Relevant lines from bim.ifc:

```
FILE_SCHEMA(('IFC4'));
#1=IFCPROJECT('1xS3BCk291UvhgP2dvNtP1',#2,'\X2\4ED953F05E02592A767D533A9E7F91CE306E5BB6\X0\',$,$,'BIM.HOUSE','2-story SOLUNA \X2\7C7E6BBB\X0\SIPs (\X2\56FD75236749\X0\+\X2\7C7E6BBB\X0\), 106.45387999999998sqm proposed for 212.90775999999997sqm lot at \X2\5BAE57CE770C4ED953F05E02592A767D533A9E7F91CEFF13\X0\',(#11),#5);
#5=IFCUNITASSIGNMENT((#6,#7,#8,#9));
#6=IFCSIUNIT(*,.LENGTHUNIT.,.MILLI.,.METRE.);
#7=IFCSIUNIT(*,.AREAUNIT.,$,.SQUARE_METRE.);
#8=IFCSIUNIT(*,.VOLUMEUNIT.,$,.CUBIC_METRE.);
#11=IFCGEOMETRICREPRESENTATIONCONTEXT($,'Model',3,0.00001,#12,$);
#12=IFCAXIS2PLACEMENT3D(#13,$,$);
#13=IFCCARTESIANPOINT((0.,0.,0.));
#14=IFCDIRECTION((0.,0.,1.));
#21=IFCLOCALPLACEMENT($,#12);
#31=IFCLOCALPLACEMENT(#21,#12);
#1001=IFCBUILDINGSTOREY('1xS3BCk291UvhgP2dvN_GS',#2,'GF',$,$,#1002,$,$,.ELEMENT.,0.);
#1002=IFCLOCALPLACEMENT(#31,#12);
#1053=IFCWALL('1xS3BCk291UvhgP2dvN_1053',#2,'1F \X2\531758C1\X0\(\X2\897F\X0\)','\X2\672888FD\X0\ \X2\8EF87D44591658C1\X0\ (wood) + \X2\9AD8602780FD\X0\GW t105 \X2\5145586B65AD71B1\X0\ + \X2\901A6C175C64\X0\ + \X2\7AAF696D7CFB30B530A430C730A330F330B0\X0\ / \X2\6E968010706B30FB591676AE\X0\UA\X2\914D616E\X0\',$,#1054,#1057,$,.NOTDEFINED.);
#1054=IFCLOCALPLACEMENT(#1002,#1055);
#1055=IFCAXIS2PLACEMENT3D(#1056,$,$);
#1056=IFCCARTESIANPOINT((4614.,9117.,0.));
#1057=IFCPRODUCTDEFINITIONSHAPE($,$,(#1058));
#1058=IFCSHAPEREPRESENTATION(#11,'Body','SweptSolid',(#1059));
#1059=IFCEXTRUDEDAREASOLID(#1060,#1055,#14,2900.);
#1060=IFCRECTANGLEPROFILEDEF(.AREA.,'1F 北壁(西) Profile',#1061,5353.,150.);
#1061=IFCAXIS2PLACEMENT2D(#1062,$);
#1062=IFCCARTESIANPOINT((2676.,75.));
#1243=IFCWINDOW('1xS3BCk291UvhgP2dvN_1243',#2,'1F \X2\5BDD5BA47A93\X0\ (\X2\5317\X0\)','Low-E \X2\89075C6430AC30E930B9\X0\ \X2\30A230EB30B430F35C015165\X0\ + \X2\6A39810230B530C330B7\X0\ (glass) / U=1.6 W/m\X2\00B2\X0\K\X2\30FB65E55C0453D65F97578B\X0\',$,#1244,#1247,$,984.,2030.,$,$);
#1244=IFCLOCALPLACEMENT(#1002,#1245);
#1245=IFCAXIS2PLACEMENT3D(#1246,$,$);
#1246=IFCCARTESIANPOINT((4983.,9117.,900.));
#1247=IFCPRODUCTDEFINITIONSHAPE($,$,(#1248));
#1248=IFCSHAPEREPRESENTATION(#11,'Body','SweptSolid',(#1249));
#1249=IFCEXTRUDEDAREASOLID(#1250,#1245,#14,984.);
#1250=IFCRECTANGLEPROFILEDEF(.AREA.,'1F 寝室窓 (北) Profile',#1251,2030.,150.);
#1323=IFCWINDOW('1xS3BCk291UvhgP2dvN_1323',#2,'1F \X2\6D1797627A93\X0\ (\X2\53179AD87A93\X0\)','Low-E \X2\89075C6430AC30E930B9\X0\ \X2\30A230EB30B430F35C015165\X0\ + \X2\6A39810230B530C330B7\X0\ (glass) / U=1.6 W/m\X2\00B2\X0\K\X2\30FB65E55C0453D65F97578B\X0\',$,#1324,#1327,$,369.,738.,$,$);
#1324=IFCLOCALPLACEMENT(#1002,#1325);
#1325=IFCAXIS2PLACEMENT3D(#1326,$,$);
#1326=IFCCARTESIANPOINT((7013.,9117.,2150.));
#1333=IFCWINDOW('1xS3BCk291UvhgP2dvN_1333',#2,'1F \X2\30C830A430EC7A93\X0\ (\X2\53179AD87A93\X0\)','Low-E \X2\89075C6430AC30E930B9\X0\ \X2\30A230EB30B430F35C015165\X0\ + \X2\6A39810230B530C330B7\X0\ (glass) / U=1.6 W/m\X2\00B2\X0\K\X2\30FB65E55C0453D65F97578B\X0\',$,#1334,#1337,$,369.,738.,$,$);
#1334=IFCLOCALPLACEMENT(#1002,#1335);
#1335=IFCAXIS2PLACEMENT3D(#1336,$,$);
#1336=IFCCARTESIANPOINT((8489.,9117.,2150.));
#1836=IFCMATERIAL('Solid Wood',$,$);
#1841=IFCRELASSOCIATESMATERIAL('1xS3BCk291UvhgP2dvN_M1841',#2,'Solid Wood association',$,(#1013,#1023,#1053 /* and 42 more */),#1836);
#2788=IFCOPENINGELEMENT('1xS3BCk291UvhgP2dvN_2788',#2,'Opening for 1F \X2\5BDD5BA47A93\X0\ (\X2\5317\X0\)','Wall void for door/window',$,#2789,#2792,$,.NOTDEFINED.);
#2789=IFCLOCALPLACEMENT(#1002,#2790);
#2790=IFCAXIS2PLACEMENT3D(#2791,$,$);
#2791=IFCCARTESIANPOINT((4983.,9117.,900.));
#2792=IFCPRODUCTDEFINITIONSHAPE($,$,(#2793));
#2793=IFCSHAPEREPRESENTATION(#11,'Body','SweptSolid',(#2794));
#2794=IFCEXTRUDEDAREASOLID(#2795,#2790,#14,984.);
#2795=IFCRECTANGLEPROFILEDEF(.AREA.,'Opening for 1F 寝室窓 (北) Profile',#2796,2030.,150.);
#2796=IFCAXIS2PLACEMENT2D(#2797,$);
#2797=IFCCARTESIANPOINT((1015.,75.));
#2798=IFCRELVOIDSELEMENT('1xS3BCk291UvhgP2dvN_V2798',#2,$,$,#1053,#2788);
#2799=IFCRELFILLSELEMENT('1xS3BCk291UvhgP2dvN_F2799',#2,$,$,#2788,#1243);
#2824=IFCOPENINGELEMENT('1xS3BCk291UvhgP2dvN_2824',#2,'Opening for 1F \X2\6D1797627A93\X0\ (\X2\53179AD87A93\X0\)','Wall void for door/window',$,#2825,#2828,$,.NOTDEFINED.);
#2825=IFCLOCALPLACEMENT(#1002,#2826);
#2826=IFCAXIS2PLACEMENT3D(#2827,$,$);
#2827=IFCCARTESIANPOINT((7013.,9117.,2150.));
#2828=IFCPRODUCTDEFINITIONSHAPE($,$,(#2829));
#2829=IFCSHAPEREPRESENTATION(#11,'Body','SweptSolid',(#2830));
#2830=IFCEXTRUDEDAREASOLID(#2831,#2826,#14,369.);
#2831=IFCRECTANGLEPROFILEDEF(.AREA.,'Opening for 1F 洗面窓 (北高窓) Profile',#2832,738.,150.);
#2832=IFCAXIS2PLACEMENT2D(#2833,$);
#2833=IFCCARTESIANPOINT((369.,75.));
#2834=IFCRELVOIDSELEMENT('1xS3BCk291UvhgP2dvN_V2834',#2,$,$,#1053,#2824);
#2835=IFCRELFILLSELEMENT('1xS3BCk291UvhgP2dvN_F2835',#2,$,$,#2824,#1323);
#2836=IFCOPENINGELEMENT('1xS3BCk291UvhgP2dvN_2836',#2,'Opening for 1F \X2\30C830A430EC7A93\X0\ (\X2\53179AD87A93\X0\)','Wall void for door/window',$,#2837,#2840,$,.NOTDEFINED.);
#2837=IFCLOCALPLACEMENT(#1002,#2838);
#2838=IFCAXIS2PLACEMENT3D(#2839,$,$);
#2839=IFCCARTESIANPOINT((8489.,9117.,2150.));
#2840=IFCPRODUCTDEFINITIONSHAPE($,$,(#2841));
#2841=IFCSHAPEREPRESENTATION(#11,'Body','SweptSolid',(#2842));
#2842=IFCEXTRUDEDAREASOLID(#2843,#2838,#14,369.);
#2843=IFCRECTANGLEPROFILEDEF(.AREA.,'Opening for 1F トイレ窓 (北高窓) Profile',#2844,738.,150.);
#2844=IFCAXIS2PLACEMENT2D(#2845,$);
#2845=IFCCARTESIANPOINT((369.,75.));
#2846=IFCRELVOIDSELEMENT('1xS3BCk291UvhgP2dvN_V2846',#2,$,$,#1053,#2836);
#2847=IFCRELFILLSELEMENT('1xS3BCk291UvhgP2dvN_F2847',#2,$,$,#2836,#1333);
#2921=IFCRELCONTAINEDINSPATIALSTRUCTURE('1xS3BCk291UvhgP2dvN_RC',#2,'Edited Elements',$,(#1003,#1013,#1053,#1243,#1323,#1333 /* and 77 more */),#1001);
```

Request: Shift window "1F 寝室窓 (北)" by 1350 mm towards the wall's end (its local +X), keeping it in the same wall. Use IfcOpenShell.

```python
import ifcopenshell
import ifcopenshell.api.geometry
import ifcopenshell.util.placement
import ifcopenshell.util.unit

model = ifcopenshell.open("bim.ifc")
unit_scale = ifcopenshell.util.unit.calculate_unit_scale(model)

window = model.by_guid("1xS3BCk291UvhgP2dvN_1243")
opening = window.FillsVoids[0].RelatingOpeningElement
wall = opening.VoidsElements[0].RelatingBuildingElement

wall_matrix = ifcopenshell.util.placement.get_local_placement(wall.ObjectPlacement)
shift = wall_matrix[:3, 0] * 1.35 / unit_scale
before = ifcopenshell.util.placement.get_local_placement(window.ObjectPlacement)[:3, 3].copy()

# The window is not placed relative to its opening, so move both.
for product in (opening, window):
    matrix = ifcopenshell.util.placement.get_local_placement(product.ObjectPlacement)
    matrix[:3, 3] += shift
    ifcopenshell.api.geometry.edit_object_placement(model, product=product, matrix=matrix, is_si=False)

after = ifcopenshell.util.placement.get_local_placement(window.ObjectPlacement)[:3, 3]
print("window moved by", (after - before).round(3) + 0.0)

model.write("bim_edited.ifc")
```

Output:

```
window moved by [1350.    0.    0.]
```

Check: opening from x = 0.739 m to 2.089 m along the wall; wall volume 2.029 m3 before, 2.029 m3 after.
